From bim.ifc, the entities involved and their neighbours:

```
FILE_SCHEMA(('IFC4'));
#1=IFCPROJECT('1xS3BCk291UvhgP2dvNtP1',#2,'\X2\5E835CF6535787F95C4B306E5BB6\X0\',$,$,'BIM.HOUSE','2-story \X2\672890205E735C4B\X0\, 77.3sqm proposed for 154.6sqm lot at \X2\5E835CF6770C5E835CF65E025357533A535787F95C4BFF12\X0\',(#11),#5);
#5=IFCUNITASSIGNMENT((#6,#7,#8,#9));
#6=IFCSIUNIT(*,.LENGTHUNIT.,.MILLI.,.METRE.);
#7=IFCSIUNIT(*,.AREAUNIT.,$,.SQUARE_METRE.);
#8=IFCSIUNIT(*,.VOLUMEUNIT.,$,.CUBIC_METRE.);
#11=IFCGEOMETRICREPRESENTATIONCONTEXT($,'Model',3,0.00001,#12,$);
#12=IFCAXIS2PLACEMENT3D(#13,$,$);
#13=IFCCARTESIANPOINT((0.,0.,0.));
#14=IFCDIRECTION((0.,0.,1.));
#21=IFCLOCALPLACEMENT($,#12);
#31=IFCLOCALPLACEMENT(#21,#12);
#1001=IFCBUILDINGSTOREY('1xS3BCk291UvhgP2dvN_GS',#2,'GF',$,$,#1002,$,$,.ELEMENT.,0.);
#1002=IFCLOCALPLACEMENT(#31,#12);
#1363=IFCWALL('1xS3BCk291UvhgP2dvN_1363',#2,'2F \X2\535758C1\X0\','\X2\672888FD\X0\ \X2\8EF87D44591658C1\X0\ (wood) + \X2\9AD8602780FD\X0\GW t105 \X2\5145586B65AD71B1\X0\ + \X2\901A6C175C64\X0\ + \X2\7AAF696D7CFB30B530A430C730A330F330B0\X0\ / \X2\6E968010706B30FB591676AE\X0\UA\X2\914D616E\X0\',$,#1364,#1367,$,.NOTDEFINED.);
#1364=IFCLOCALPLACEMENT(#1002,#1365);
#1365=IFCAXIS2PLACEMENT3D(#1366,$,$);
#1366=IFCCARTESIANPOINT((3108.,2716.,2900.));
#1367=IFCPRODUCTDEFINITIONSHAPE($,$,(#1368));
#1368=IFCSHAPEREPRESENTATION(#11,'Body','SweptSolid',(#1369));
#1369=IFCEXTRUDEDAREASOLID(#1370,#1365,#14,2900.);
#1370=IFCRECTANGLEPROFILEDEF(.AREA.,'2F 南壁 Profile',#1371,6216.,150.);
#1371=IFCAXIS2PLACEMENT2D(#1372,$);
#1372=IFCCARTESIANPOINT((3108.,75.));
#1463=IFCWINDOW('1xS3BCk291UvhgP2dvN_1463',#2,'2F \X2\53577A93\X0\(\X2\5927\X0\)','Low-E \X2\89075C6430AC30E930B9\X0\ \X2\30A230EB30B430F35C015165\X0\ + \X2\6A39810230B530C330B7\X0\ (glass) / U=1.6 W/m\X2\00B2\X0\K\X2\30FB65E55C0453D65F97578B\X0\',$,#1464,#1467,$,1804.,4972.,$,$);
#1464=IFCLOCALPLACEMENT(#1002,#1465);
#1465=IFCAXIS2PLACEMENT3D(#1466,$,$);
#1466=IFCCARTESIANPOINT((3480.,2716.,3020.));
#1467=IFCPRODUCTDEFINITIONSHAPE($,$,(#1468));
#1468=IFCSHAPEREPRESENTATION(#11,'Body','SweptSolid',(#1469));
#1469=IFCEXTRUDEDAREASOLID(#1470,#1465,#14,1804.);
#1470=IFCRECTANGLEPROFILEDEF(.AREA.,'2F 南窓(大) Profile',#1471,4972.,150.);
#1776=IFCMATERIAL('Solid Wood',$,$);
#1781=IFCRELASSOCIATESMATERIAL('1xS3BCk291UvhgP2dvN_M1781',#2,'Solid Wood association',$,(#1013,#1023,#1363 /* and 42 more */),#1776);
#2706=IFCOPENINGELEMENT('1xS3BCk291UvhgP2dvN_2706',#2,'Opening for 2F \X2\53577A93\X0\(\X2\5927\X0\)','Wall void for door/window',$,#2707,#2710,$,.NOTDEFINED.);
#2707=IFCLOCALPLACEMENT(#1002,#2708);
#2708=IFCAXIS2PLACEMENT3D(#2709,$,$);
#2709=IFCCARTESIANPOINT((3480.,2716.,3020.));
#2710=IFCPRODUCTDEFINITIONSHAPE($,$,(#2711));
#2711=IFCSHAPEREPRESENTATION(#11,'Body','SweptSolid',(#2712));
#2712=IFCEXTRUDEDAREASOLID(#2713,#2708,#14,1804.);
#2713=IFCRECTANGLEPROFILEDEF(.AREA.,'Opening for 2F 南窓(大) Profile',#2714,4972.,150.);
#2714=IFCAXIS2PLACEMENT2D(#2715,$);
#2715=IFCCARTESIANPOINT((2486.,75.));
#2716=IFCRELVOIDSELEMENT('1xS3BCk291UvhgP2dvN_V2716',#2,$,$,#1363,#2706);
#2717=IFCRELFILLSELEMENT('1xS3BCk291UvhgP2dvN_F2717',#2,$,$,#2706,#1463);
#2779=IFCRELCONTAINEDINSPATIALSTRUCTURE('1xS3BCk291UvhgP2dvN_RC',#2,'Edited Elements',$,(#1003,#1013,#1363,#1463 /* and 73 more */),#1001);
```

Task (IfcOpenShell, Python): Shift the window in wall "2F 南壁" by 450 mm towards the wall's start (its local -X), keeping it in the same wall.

```python
import ifcopenshell
import ifcopenshell.api.geometry
import ifcopenshell.util.placement

model = ifcopenshell.open("bim.ifc")

window = model.by_guid("1xS3BCk291UvhgP2dvN_1463")
opening = window.FillsVoids[0].RelatingOpeningElement
wall = opening.VoidsElements[0].RelatingBuildingElement

wall_matrix = ifcopenshell.util.placement.get_local_placement(wall.ObjectPlacement)
shift = wall_matrix[:3, 0] * -450.0
before = ifcopenshell.util.placement.get_local_placement(window.ObjectPlacement)[:3, 3].copy()

# The window is not placed relative to its opening, so move both.
for product in (opening, window):
    matrix = ifcopenshell.util.placement.get_local_placement(product.ObjectPlacement)
    matrix[:3, 3] += shift
    ifcopenshell.api.geometry.edit_object_placement(model, product=product, matrix=matrix, is_si=False)

after = ifcopenshell.util.placement.get_local_placement(window.ObjectPlacement)[:3, 3]
print("window moved by", (after - before).round(3) + 0.0)

model.write("bim_rev.ifc")
```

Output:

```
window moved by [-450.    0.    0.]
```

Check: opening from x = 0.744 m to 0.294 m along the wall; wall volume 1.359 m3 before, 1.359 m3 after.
